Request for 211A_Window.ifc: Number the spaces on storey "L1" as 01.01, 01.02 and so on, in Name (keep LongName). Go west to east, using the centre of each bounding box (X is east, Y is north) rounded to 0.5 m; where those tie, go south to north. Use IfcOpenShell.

First a look at what the model holds.

```python
import ifcopenshell
import ifcopenshell.util.element
import ifcopenshell.util.placement

model = ifcopenshell.open("211A_Window.ifc")
print(model.schema)
storey = next(s for s in model.by_type("IfcBuildingStorey") if s.Name == "L1")
spaces = [e for e in ifcopenshell.util.element.get_decomposition(storey) if e.is_a("IfcSpace")]
for e in sorted(spaces, key=lambda e: e.id()):
    origin = ifcopenshell.util.placement.get_local_placement(e.ObjectPlacement)[:3, 3]
    print(e.id(), e.Name, e.LongName, origin.round(2) + 0.0, sep=" | ")
```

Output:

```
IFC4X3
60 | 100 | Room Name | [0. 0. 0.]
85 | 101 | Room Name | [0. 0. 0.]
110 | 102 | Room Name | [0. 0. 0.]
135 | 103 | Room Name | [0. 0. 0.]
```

```python
import ifcopenshell
import ifcopenshell.geom
import ifcopenshell.util.element
import ifcopenshell.util.shape

model = ifcopenshell.open("211A_Window.ifc")
settings = ifcopenshell.geom.settings()
settings.set("use-world-coords", True)


def centre(element):
    shape = ifcopenshell.geom.create_shape(settings, element)
    return ifcopenshell.util.shape.get_bbox_centroid(shape.geometry)


storey = next(s for s in model.by_type("IfcBuildingStorey") if s.Name == "L1")
spaces = [e for e in ifcopenshell.util.element.get_decomposition(storey) if e.is_a("IfcSpace")]

# Insertion points can sit at a corner or the storey origin, so sort by the geometry (in metres).
centres = {e: centre(e) for e in spaces}
spaces.sort(key=lambda e: (round(centres[e][0] / 0.5), centres[e][1]))

for i, e in enumerate(spaces, start=1):
    number = f"01.{i:02d}"
    e.Name = number
    print(e.id(), number)

model.write("211A_Window_updated.ifc")
```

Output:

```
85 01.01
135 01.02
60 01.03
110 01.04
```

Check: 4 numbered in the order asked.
